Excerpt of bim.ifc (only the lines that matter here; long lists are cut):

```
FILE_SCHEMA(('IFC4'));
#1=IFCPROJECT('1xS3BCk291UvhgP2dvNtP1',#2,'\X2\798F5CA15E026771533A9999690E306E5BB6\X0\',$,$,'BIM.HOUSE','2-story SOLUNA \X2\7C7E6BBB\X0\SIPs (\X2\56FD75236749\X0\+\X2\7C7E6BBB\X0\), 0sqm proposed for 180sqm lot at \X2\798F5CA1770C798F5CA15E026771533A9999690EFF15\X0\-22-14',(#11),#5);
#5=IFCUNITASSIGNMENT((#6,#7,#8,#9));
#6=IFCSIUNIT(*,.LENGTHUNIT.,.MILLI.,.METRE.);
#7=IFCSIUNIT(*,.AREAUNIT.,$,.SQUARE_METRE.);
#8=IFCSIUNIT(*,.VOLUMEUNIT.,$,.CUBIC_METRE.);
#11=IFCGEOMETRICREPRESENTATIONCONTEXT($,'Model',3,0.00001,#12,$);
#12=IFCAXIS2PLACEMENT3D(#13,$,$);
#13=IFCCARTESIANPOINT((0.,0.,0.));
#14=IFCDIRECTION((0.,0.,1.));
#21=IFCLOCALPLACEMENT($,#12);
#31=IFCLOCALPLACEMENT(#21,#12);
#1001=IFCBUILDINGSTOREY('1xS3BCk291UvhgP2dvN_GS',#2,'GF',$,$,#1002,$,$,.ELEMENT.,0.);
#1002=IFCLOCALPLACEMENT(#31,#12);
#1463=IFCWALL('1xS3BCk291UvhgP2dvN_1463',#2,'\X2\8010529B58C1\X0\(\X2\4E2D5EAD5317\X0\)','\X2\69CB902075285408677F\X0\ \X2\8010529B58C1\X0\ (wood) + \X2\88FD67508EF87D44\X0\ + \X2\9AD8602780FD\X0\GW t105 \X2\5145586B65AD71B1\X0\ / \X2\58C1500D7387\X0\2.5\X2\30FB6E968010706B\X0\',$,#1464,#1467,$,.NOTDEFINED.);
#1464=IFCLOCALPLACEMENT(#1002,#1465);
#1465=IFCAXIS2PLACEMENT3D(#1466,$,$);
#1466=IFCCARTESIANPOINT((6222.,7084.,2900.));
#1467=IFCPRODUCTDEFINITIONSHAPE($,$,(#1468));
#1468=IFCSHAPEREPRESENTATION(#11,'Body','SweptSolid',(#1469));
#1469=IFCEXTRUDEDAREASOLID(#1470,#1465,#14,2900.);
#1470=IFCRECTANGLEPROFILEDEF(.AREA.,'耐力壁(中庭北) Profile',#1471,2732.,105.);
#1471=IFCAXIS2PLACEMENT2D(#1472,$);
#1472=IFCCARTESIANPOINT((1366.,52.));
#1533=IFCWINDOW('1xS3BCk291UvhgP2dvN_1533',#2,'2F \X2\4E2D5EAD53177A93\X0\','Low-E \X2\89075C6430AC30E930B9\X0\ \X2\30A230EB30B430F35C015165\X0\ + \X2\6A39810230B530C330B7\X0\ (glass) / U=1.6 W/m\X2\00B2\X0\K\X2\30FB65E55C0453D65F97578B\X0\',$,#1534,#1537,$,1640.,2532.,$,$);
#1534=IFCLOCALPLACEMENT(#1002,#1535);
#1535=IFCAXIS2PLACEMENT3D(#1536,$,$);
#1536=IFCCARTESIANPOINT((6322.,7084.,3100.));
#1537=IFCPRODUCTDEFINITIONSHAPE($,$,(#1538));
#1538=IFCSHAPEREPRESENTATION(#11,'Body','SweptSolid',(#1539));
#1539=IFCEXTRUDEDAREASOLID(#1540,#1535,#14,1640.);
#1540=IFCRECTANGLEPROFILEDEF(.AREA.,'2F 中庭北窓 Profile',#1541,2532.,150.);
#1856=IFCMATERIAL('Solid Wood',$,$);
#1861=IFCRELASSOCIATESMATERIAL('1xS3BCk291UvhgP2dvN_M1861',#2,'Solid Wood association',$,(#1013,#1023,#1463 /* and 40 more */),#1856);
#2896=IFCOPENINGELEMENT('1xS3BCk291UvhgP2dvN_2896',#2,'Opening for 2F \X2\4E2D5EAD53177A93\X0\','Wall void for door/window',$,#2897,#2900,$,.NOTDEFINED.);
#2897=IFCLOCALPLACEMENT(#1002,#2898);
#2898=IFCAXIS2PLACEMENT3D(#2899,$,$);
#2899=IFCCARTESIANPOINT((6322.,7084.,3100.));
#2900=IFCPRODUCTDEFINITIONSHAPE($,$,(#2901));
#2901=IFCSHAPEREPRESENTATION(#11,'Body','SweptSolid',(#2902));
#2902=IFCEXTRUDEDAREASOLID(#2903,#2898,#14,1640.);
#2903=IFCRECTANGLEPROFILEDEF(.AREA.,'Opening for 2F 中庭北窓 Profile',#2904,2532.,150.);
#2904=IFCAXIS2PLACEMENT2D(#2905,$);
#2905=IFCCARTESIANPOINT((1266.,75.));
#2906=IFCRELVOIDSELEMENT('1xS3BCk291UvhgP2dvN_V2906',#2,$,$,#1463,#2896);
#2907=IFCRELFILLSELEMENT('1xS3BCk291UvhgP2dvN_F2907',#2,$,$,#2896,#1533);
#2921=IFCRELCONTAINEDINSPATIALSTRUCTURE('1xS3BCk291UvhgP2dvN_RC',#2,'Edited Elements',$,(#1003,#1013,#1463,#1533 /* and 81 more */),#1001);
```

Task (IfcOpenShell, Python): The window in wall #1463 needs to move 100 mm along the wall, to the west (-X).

```python
import ifcopenshell
import ifcopenshell.api.geometry
import ifcopenshell.util.placement
import ifcopenshell.util.unit

model = ifcopenshell.open("bim.ifc")
unit_scale = ifcopenshell.util.unit.calculate_unit_scale(model)

window = model.by_id(1533)
opening = window.FillsVoids[0].RelatingOpeningElement
wall = opening.VoidsElements[0].RelatingBuildingElement

wall_matrix = ifcopenshell.util.placement.get_local_placement(wall.ObjectPlacement)
shift = wall_matrix[:3, 0] * -0.1 / unit_scale
before = ifcopenshell.util.placement.get_local_placement(window.ObjectPlacement)[:3, 3].copy()

# The window is not placed relative to its opening, so move both.
for product in (opening, window):
    matrix = ifcopenshell.util.placement.get_local_placement(product.ObjectPlacement)
    matrix[:3, 3] += shift
    ifcopenshell.api.geometry.edit_object_placement(model, product=product, matrix=matrix, is_si=False)

after = ifcopenshell.util.placement.get_local_placement(window.ObjectPlacement)[:3, 3]
print("window moved by", (after - before).round(3) + 0.0)

model.write("bim_v2.ifc")
```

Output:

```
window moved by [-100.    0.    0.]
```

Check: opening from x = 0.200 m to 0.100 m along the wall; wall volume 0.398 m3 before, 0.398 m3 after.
